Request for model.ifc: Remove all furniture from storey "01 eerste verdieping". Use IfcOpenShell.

First a look at what the model holds.

```python
import ifcopenshell
import ifcopenshell.util.element

model = ifcopenshell.open("model.ifc")
print(model.schema)
storey = next(s for s in model.by_type("IfcBuildingStorey") if s.Name == "01 eerste verdieping")
furniture = [e for e in ifcopenshell.util.element.get_decomposition(storey) if e.is_a("IfcFurnishingElement")]
seen = {}
for e in furniture:
    element_type = ifcopenshell.util.element.get_type(e)
    name = element_type.Name if element_type not in (None, e) else None
    seen[name] = seen.get(name, 0) + 1
for name, count in sorted(seen.items(), key=str):
    print(count, "x", name)
```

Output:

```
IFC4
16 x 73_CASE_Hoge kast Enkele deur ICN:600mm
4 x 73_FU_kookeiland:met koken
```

```python
import ifcopenshell
import ifcopenshell.api.root
import ifcopenshell.util.element

model = ifcopenshell.open("model.ifc")

storey = next(s for s in model.by_type("IfcBuildingStorey") if s.Name == "01 eerste verdieping")
furniture = [e for e in ifcopenshell.util.element.get_decomposition(storey) if e.is_a("IfcFurnishingElement")]

for e in furniture:
    ifcopenshell.api.root.remove_product(model, product=e)
print(len(furniture), "removed")

model.write("model_updated.ifc")
```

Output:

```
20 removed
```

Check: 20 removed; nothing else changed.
